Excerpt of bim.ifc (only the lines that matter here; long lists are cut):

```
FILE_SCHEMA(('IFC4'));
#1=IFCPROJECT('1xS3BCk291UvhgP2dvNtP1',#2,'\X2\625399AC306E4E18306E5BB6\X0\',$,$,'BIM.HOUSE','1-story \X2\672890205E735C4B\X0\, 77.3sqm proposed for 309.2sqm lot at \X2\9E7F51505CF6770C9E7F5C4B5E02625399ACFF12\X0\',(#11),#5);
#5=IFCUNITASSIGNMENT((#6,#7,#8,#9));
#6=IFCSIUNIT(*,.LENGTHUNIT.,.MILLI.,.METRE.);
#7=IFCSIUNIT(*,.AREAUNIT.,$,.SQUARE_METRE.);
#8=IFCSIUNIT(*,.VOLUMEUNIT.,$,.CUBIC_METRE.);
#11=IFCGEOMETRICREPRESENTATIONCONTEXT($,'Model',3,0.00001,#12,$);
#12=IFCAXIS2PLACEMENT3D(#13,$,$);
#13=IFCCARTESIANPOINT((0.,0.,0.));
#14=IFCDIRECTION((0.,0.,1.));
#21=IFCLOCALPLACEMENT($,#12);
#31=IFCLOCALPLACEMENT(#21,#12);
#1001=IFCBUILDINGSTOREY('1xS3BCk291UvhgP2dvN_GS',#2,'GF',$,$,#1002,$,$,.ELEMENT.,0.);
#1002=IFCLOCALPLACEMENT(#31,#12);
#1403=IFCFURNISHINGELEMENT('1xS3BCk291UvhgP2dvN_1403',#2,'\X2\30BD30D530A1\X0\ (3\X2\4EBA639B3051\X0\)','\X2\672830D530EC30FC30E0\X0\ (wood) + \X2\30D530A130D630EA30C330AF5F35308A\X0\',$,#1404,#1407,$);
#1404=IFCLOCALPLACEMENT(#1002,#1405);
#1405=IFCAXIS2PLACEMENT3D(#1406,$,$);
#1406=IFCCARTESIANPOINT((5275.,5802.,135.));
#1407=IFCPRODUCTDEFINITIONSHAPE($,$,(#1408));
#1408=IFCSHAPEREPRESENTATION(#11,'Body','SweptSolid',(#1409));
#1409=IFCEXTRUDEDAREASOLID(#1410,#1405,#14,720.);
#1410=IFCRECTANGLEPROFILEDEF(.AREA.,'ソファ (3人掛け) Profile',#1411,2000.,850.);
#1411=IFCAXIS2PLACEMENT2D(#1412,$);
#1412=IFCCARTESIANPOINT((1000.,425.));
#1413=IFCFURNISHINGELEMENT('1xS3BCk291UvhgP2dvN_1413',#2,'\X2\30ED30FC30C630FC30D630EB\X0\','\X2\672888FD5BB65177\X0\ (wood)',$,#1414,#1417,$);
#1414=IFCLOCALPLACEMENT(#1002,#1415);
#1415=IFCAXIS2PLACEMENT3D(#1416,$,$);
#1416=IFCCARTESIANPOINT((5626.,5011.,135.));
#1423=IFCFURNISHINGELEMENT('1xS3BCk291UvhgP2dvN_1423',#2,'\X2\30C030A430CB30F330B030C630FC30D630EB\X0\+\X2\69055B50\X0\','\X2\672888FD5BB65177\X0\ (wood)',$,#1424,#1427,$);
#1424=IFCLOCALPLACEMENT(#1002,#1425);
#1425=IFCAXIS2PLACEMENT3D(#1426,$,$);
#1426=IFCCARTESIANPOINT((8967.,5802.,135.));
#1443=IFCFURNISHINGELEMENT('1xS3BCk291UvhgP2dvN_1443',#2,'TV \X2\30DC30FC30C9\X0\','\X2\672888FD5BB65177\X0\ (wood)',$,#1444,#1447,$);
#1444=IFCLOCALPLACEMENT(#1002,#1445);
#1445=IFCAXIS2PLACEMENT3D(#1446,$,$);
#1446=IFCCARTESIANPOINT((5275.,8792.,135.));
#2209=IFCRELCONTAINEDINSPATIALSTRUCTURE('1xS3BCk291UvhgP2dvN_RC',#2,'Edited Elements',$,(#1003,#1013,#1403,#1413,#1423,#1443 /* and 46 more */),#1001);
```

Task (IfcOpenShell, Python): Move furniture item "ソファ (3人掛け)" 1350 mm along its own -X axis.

```python
import ifcopenshell
import ifcopenshell.api.geometry
import ifcopenshell.util.placement
import ifcopenshell.util.unit

model = ifcopenshell.open("bim.ifc")
unit_scale = ifcopenshell.util.unit.calculate_unit_scale(model)

item = model.by_guid("1xS3BCk291UvhgP2dvN_1403")
matrix = ifcopenshell.util.placement.get_local_placement(item.ObjectPlacement)
matrix[:3, 3] -= matrix[:3, 0] * 1.35 / unit_scale
ifcopenshell.api.geometry.edit_object_placement(model, product=item, matrix=matrix, is_si=False)

print(ifcopenshell.util.placement.get_local_placement(item.ObjectPlacement).round(3) + 0.0)

model.write("bim_updated.ifc")
```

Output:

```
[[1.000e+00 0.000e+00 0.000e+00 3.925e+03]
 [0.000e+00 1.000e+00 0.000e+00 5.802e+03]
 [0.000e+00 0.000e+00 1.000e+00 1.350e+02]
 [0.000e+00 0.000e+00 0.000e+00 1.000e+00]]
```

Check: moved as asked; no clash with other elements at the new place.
